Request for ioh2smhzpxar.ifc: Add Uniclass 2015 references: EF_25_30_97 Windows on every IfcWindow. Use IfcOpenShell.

First a look at what the model holds.

```python
import ifcopenshell

model = ifcopenshell.open("ioh2smhzpxar.ifc")
print(model.schema)
print("classifications:", [c.Name for c in model.by_type("IfcClassification")])
for ifc_class in ("IfcDoor", "IfcRoof", "IfcStair", "IfcWall", "IfcWindow"):
    print(ifc_class, len(model.by_type(ifc_class)))
```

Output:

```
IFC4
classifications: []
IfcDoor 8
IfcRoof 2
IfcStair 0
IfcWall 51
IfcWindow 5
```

```python
import ifcopenshell
import ifcopenshell.api.classification

model = ifcopenshell.open("ioh2smhzpxar.ifc")

system = ifcopenshell.api.classification.add_classification(model, classification="Uniclass 2015")

codes = {
    "IfcWindow": ("EF_25_30_97", "Windows"),
}
for ifc_class, (code, name) in codes.items():
    products = model.by_type(ifc_class)
    ifcopenshell.api.classification.add_reference(
        model, products=products, classification=system, identification=code, name=name
    )
    print(code, len(products))

model.write("ioh2smhzpxar_edited.ifc")
```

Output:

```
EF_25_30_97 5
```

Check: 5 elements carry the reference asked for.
